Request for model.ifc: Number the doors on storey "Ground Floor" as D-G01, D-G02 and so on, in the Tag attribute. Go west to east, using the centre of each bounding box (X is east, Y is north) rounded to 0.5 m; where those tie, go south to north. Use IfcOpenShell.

First a look at what the model holds.

```python
import ifcopenshell
import ifcopenshell.util.element
import ifcopenshell.util.placement

model = ifcopenshell.open("model.ifc")
print(model.schema)
storey = next(s for s in model.by_type("IfcBuildingStorey") if s.Name == "Ground Floor")
doors = [e for e in ifcopenshell.util.element.get_decomposition(storey) if e.is_a("IfcDoor")]
for e in sorted(doors, key=lambda e: e.id()):
    origin = ifcopenshell.util.placement.get_local_placement(e.ObjectPlacement)[:3, 3]
    print(e.id(), e.Tag, e.Name, origin.round(2) + 0.0, sep=" | ")
```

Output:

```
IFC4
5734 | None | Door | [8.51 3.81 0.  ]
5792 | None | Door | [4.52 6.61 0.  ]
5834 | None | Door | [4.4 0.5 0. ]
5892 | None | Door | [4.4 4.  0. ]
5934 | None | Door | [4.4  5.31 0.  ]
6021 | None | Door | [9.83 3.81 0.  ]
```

```python
import ifcopenshell
import ifcopenshell.geom
import ifcopenshell.util.element
import ifcopenshell.util.shape

model = ifcopenshell.open("model.ifc")
settings = ifcopenshell.geom.settings()
settings.set("use-world-coords", True)


def centre(element):
    shape = ifcopenshell.geom.create_shape(settings, element)
    return ifcopenshell.util.shape.get_bbox_centroid(shape.geometry)


storey = next(s for s in model.by_type("IfcBuildingStorey") if s.Name == "Ground Floor")
doors = [e for e in ifcopenshell.util.element.get_decomposition(storey) if e.is_a("IfcDoor")]

# Insertion points can sit at a corner or the storey origin, so sort by the geometry (in metres).
centres = {e: centre(e) for e in doors}
doors.sort(key=lambda e: (round(centres[e][0] / 0.5), centres[e][1]))

for i, e in enumerate(doors, start=1):
    number = f"D-G{i:02d}"
    e.Tag = number
    print(e.id(), number)

model.write("model_updated.ifc")
```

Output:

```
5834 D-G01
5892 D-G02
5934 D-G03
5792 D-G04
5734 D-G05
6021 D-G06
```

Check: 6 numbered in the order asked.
